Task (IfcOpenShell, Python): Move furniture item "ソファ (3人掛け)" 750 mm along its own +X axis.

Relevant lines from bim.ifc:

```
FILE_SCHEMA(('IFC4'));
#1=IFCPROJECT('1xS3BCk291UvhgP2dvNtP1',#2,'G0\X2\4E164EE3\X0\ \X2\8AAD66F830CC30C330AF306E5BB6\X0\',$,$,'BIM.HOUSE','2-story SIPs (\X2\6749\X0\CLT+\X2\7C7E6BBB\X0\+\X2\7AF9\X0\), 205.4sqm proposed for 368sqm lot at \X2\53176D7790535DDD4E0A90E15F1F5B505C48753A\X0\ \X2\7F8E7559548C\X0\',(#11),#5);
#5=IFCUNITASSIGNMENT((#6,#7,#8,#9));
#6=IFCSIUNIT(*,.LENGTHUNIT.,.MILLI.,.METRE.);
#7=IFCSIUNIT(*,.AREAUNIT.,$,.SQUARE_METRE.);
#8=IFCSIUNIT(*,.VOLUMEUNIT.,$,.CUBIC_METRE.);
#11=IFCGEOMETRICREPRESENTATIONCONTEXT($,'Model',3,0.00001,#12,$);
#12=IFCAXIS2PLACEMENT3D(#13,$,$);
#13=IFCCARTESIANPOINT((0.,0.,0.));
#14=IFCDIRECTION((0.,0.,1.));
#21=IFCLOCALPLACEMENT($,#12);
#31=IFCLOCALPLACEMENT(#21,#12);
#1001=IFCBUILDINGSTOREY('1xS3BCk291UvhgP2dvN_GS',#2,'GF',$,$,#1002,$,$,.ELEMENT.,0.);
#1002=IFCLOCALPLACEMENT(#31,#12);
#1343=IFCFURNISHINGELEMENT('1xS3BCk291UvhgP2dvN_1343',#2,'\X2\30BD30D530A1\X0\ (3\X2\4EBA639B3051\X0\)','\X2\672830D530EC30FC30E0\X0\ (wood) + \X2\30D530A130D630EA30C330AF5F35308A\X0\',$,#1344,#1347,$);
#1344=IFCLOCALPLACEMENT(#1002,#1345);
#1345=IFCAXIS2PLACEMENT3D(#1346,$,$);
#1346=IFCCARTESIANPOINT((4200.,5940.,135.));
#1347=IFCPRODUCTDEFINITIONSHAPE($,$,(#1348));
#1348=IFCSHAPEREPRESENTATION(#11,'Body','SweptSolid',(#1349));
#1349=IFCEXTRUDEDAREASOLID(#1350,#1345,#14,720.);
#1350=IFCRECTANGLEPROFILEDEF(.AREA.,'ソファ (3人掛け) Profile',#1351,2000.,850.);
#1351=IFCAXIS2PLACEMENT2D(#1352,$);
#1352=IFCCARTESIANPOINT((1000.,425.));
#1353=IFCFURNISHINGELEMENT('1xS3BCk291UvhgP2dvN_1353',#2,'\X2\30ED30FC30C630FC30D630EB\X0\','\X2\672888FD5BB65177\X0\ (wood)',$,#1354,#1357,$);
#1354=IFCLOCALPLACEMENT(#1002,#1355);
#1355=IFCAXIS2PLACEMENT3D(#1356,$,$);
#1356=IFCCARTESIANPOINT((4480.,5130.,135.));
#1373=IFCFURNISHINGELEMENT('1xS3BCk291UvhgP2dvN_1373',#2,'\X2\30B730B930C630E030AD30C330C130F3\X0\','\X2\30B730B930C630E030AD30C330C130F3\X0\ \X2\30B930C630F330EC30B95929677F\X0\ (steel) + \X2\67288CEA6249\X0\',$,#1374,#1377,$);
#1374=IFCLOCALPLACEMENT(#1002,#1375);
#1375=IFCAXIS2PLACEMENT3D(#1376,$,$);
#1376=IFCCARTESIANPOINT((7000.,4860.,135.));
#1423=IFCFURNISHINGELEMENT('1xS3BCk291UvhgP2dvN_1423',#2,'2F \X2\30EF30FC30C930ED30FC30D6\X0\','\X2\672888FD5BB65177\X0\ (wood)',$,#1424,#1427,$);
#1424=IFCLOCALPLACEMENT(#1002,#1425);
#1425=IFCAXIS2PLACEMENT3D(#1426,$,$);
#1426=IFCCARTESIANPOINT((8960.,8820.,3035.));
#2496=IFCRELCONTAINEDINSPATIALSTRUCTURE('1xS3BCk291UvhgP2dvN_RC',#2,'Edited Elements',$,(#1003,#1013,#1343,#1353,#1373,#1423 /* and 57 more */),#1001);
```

```python
import ifcopenshell
import ifcopenshell.api.geometry
import ifcopenshell.util.placement
import ifcopenshell.util.unit

model = ifcopenshell.open("bim.ifc")
unit_scale = ifcopenshell.util.unit.calculate_unit_scale(model)

item = model.by_guid("1xS3BCk291UvhgP2dvN_1343")
matrix = ifcopenshell.util.placement.get_local_placement(item.ObjectPlacement)
matrix[:3, 3] += matrix[:3, 0] * 0.75 / unit_scale
ifcopenshell.api.geometry.edit_object_placement(model, product=item, matrix=matrix, is_si=False)

print(ifcopenshell.util.placement.get_local_placement(item.ObjectPlacement).round(3) + 0.0)

model.write("bim_rev.ifc")
```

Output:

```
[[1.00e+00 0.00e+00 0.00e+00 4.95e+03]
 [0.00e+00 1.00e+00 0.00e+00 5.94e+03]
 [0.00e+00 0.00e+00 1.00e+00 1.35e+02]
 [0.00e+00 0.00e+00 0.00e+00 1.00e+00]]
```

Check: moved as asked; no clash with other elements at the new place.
